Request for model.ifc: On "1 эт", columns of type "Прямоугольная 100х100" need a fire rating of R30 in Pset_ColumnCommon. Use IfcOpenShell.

First a look at what the model holds.

```python
import ifcopenshell
import ifcopenshell.util.element

model = ifcopenshell.open("model.ifc")
print(model.schema)
storey = next(s for s in model.by_type("IfcBuildingStorey") if s.Name == "1 эт")
columns = [e for e in ifcopenshell.util.element.get_decomposition(storey) if e.is_a("IfcColumn")]
seen = {}
for e in columns:
    element_type = ifcopenshell.util.element.get_type(e)
    key = (element_type.Name if element_type != e and element_type else None, ifcopenshell.util.element.get_pset(e, "Pset_ColumnCommon", "FireRating"))
    seen[key] = seen.get(key, 0) + 1
for (name, value), count in sorted(seen.items(), key=str):
    print(count, "x", name, "|", value)
```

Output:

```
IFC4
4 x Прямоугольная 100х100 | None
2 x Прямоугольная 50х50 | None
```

```python
import ifcopenshell
import ifcopenshell.api.pset
import ifcopenshell.util.element

model = ifcopenshell.open("model.ifc")

storey = next(s for s in model.by_type("IfcBuildingStorey") if s.Name == "1 эт")
columns = [e for e in ifcopenshell.util.element.get_decomposition(storey) if e.is_a("IfcColumn")]

count = 0
for e in columns:
    element_type = ifcopenshell.util.element.get_type(e)
    if element_type in (None, e) or element_type.Name != "Прямоугольная 100х100":
        continue
    # add_pset returns the element's existing set when there is one.
    pset = ifcopenshell.api.pset.add_pset(model, product=e, name="Pset_ColumnCommon")
    ifcopenshell.api.pset.edit_pset(model, pset=pset, properties={"FireRating": "R30"})
    count += 1

print(count, "columns updated")

model.write("model_v2.ifc")
```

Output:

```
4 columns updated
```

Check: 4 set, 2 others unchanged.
